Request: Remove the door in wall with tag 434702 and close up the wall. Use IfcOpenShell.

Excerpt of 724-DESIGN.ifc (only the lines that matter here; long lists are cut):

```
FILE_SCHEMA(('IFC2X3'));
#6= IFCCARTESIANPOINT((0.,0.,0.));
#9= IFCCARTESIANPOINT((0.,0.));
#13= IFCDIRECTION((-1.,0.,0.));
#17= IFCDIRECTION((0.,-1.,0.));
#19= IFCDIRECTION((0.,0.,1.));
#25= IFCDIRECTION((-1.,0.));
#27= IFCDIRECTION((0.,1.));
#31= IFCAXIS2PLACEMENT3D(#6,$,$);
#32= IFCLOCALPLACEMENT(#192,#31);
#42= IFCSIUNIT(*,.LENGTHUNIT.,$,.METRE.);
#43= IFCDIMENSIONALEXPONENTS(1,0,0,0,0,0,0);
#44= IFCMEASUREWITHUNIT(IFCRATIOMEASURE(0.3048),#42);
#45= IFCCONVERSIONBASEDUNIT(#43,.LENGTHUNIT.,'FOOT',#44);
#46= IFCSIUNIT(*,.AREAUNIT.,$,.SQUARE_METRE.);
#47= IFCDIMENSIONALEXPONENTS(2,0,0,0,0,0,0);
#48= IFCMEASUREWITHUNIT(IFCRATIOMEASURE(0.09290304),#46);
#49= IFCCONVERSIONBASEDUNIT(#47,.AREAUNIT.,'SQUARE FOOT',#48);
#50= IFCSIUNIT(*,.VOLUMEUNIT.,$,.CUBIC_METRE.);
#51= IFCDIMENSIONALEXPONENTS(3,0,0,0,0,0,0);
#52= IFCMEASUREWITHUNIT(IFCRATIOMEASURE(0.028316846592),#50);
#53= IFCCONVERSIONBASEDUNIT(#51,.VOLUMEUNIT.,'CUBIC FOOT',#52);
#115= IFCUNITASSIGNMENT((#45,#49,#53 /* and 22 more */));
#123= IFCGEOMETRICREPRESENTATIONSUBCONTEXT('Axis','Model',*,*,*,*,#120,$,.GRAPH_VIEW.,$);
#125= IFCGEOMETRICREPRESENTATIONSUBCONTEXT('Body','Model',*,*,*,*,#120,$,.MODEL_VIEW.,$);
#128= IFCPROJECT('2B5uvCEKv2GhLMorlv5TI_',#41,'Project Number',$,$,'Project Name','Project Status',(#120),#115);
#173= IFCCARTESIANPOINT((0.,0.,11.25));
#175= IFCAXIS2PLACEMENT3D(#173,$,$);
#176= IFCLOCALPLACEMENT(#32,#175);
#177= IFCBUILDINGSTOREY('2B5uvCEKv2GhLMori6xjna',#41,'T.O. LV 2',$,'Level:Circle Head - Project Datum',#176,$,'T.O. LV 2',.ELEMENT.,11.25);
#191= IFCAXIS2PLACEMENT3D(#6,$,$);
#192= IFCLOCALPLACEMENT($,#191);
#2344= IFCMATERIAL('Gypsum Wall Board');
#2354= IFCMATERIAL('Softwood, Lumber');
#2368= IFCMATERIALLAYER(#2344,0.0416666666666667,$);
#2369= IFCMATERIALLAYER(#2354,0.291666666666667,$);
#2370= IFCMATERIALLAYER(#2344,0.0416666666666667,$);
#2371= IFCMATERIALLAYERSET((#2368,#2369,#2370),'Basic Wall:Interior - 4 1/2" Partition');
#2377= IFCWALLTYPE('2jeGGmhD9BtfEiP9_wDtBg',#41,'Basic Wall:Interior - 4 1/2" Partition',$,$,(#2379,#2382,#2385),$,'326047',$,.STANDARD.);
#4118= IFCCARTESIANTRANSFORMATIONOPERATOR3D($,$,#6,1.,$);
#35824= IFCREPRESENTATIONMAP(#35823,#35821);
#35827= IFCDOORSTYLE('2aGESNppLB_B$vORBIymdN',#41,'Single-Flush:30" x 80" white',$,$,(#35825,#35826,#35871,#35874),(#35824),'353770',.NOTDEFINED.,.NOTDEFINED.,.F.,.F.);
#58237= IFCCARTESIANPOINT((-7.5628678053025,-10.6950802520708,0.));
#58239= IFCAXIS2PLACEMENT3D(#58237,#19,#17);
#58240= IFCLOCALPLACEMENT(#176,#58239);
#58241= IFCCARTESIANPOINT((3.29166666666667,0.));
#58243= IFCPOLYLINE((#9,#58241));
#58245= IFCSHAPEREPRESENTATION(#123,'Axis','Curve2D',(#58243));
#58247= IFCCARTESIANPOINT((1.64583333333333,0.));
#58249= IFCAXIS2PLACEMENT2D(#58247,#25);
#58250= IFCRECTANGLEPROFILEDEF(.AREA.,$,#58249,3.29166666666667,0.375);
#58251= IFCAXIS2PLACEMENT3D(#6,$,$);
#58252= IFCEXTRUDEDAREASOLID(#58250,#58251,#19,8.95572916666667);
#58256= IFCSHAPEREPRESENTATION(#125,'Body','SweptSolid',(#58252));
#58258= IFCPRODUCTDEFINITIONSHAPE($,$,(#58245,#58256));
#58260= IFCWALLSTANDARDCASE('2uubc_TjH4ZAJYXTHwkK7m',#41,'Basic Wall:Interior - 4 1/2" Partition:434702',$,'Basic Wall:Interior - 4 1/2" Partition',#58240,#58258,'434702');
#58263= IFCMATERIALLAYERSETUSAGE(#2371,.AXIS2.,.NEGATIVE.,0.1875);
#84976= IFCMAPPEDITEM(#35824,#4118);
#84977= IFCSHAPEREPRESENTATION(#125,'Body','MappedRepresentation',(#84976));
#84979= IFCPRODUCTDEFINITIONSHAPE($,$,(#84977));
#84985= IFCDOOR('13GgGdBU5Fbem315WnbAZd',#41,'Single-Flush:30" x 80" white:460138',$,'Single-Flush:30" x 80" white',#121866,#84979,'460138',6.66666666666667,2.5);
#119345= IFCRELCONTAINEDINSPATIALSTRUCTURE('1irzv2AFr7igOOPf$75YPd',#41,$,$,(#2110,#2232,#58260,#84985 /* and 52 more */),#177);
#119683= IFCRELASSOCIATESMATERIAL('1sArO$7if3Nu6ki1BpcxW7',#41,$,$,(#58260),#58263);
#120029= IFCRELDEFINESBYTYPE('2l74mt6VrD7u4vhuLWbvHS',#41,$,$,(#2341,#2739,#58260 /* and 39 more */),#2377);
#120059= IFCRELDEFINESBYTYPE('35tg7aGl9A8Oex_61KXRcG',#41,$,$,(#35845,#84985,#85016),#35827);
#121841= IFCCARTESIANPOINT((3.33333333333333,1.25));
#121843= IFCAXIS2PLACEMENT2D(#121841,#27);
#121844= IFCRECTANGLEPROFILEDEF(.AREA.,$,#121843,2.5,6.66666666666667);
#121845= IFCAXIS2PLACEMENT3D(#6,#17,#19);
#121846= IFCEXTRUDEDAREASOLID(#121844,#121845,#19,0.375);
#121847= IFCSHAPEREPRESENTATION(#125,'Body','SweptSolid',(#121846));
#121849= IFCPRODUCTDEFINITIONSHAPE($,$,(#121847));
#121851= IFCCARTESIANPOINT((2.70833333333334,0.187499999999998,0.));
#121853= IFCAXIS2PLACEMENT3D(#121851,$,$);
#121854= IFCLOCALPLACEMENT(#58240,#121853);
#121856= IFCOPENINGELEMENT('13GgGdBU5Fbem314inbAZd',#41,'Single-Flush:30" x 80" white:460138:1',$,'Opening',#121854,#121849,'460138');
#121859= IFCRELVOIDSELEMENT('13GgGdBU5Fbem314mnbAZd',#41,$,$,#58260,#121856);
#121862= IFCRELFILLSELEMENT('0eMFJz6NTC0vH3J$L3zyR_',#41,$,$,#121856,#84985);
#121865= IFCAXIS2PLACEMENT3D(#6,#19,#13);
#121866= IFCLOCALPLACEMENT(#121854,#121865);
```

```python
import ifcopenshell
import ifcopenshell.api.feature
import ifcopenshell.api.root
import ifcopenshell.geom
import ifcopenshell.util.shape

model = ifcopenshell.open("724-DESIGN.ifc")
settings = ifcopenshell.geom.settings()


def volume(element):
    """Net volume in cubic metres, openings subtracted."""
    shape = ifcopenshell.geom.create_shape(settings, element)
    return ifcopenshell.util.shape.get_volume(shape.geometry)


door = model.by_id(84985)
opening = door.FillsVoids[0].RelatingOpeningElement
wall = opening.VoidsElements[0].RelatingBuildingElement
before = volume(wall)

ifcopenshell.api.root.remove_product(model, product=door)
ifcopenshell.api.feature.remove_feature(model, feature=opening)

after = volume(wall)

print(f"wall volume {before:.3f} -> {after:.3f} m3")

model.write("724-DESIGN_edited.ifc")
```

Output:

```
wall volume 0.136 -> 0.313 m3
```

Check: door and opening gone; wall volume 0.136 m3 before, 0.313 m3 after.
